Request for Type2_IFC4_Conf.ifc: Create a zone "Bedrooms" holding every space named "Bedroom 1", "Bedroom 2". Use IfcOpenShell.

First a look at what the model holds.

```python
import ifcopenshell

model = ifcopenshell.open("Type2_IFC4_Conf.ifc")
print(model.schema)
seen = {}
for space in model.by_type("IfcSpace"):
    seen[space.LongName] = seen.get(space.LongName, 0) + 1
for name, count in sorted(seen.items(), key=str):
    print(count, "x", name)
print("zones:", [z.Name for z in model.by_type("IfcZone")][:20])
```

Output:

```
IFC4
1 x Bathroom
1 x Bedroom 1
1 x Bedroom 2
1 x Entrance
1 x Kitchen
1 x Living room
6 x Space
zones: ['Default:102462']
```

```python
import ifcopenshell
import ifcopenshell.api.group
import ifcopenshell.api.root

model = ifcopenshell.open("Type2_IFC4_Conf.ifc")

names = {"Bedroom 1", "Bedroom 2"}
spaces = [s for s in model.by_type("IfcSpace") if s.LongName in names]

zone = ifcopenshell.api.root.create_entity(model, ifc_class="IfcZone", name="Bedrooms")
ifcopenshell.api.group.assign_group(model, products=spaces, group=zone)
print(len(spaces), "spaces in", zone.Name)

model.write("Type2_IFC4_Conf_updated.ifc")
```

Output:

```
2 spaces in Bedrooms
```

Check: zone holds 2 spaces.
